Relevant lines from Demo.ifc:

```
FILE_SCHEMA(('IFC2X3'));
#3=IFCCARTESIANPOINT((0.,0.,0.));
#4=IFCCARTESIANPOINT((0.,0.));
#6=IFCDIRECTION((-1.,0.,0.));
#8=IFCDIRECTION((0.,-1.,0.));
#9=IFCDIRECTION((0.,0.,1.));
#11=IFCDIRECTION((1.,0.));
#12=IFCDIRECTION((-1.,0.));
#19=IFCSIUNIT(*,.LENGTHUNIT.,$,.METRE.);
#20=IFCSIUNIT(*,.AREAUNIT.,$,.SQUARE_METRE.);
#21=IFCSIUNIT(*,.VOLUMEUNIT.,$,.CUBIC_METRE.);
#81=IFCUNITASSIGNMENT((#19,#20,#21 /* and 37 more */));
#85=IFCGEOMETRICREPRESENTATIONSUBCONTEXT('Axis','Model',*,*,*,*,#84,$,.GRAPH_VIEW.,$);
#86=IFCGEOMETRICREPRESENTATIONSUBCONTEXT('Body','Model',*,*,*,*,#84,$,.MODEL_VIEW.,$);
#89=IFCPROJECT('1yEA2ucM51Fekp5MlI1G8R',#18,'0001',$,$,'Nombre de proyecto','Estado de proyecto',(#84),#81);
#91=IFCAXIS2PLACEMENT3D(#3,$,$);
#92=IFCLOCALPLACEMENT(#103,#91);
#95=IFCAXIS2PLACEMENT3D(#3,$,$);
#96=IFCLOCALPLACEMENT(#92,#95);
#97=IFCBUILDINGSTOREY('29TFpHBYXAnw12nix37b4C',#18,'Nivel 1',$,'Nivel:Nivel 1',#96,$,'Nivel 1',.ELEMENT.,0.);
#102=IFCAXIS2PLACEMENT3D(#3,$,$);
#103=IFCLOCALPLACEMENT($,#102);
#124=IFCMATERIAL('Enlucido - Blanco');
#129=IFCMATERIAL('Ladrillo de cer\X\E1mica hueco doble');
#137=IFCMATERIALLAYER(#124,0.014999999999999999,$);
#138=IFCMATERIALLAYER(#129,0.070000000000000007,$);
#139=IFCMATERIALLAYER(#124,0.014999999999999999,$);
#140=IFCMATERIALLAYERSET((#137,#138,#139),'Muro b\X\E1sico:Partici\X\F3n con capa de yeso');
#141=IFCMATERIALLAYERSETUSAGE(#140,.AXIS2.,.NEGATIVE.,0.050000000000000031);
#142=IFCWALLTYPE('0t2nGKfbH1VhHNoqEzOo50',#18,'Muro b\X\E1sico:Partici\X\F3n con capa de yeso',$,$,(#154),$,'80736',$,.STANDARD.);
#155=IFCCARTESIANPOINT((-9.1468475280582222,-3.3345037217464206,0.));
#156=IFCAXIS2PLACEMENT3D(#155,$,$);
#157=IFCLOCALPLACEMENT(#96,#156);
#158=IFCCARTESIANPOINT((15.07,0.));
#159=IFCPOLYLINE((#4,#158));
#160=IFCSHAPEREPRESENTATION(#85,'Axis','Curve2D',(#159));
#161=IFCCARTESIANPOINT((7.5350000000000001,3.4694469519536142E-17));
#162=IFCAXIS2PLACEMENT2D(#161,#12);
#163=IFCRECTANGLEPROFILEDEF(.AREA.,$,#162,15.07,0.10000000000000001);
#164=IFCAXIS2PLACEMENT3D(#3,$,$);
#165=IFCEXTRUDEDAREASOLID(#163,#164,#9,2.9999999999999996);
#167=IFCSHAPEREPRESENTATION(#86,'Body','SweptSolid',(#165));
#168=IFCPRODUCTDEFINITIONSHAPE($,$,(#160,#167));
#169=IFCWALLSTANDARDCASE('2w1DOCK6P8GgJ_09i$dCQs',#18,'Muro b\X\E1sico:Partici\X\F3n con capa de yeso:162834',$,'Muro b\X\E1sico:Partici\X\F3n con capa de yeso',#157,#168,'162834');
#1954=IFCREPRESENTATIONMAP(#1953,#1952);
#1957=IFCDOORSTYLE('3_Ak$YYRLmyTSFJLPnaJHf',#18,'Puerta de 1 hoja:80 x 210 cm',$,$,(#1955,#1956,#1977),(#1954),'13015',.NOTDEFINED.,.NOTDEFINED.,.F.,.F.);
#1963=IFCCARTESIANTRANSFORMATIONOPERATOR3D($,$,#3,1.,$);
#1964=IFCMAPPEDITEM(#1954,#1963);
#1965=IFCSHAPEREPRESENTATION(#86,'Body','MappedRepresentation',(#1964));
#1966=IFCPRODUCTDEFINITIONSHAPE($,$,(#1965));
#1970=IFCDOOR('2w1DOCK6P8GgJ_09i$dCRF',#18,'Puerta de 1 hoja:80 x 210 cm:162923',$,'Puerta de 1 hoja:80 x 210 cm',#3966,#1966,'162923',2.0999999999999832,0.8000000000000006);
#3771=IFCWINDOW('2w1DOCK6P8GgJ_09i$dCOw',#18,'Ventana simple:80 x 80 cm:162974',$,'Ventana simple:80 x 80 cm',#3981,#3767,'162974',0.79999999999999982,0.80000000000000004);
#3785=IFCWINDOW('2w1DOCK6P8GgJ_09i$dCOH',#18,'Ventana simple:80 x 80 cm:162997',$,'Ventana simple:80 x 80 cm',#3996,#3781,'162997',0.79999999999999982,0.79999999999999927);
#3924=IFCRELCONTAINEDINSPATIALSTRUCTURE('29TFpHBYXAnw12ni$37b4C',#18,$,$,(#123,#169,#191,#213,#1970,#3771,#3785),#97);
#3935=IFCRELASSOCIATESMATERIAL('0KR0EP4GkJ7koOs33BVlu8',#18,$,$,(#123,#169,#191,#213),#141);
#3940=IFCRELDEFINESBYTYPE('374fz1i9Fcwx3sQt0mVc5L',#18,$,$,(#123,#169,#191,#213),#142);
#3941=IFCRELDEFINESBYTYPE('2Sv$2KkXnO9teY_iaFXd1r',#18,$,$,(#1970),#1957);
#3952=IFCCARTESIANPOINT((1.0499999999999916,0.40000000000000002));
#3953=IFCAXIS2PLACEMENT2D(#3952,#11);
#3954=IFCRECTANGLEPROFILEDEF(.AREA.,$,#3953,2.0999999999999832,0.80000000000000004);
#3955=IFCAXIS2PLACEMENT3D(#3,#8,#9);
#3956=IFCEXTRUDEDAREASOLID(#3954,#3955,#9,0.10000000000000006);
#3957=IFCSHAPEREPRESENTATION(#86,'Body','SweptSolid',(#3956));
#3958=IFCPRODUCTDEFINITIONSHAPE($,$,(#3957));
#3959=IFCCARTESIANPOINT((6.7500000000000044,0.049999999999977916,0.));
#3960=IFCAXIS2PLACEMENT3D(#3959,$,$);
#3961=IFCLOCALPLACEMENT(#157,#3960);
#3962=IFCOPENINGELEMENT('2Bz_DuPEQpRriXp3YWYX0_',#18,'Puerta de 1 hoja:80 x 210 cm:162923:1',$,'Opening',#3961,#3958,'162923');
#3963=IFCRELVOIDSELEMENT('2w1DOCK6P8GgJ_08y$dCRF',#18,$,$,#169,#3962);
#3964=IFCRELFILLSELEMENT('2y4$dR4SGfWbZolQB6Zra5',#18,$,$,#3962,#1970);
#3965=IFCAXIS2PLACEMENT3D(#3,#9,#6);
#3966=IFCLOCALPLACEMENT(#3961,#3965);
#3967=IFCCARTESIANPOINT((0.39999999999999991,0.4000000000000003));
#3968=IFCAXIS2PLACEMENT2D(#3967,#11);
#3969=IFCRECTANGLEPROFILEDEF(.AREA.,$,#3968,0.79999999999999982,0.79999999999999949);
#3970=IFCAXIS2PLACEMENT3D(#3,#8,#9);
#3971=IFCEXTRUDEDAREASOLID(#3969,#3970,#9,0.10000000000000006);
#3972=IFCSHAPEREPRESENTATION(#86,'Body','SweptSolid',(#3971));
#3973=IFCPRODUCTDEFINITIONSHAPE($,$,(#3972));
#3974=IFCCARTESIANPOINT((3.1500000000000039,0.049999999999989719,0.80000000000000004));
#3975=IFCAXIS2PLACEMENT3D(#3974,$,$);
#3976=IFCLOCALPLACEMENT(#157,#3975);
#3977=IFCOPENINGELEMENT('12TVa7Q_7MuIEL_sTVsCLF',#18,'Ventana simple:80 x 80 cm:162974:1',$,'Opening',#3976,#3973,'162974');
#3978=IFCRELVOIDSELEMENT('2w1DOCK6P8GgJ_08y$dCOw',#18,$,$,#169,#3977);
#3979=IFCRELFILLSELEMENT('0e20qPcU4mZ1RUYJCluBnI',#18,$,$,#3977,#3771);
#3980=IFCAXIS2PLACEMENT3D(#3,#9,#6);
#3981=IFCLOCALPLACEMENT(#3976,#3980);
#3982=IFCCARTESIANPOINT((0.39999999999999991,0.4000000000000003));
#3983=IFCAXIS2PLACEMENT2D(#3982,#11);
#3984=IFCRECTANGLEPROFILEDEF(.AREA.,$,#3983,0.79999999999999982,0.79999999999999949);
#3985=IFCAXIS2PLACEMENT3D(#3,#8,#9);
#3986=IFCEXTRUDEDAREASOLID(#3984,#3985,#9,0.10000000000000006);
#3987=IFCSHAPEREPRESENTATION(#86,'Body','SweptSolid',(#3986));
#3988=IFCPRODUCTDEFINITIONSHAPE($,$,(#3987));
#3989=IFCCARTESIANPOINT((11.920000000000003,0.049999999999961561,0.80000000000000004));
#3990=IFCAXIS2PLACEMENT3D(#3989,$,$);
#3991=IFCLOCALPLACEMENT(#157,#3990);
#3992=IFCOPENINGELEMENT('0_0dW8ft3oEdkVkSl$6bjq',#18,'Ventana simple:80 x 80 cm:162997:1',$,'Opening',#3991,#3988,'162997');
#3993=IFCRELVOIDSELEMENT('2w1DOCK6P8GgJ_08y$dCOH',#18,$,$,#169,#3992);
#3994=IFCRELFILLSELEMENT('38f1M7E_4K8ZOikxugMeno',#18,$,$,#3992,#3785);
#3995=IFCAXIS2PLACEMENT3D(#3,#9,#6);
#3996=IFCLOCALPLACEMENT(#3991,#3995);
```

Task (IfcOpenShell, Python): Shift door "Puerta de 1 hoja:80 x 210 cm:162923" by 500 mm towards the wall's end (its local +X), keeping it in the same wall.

```python
import ifcopenshell
import ifcopenshell.api.geometry
import ifcopenshell.util.placement
import ifcopenshell.util.unit

model = ifcopenshell.open("Demo.ifc")
unit_scale = ifcopenshell.util.unit.calculate_unit_scale(model)

door = model.by_id(1970)
opening = door.FillsVoids[0].RelatingOpeningElement
wall = opening.VoidsElements[0].RelatingBuildingElement

wall_matrix = ifcopenshell.util.placement.get_local_placement(wall.ObjectPlacement)
shift = wall_matrix[:3, 0] * 0.5 / unit_scale
before = ifcopenshell.util.placement.get_local_placement(door.ObjectPlacement)[:3, 3].copy()

# The door is placed relative to its opening, so it follows when the opening moves.
matrix = ifcopenshell.util.placement.get_local_placement(opening.ObjectPlacement)
matrix[:3, 3] += shift
ifcopenshell.api.geometry.edit_object_placement(
    model, product=opening, matrix=matrix, is_si=False, should_transform_children=True
)

after = ifcopenshell.util.placement.get_local_placement(door.ObjectPlacement)[:3, 3]
print("door moved by", (after - before).round(3) + 0.0)

model.write("Demo-out.ifc")
```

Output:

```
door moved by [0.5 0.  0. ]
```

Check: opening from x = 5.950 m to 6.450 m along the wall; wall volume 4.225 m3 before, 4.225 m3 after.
